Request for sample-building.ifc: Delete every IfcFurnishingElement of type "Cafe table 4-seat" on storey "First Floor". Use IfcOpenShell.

First a look at what the model holds.

```python
import ifcopenshell
import ifcopenshell.util.element

model = ifcopenshell.open("sample-building.ifc")
print(model.schema)
storey = next(s for s in model.by_type("IfcBuildingStorey") if s.Name == "First Floor")
furniture = [e for e in ifcopenshell.util.element.get_decomposition(storey) if e.is_a("IfcFurnishingElement")]
seen = {}
for e in furniture:
    element_type = ifcopenshell.util.element.get_type(e)
    name = element_type.Name if element_type not in (None, e) else None
    seen[name] = seen.get(name, 0) + 1
for name, count in sorted(seen.items(), key=str):
    print(count, "x", name)
```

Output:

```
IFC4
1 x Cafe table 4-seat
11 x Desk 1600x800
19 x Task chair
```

```python
import ifcopenshell
import ifcopenshell.api.root
import ifcopenshell.util.element

model = ifcopenshell.open("sample-building.ifc")

storey = next(s for s in model.by_type("IfcBuildingStorey") if s.Name == "First Floor")
furniture = [e for e in ifcopenshell.util.element.get_decomposition(storey) if e.is_a("IfcFurnishingElement")]
targets = [e for e in furniture if (t := ifcopenshell.util.element.get_type(e)) not in (None, e) and t.Name == "Cafe table 4-seat"]

for e in targets:
    ifcopenshell.api.root.remove_product(model, product=e)
print(len(targets), "removed")

model.write("sample-building_rev.ifc")
```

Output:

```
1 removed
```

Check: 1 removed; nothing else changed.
